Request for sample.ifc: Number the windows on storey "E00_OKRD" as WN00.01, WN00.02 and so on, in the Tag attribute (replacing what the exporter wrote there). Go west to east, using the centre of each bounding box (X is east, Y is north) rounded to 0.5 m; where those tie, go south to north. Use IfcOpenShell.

First a look at what the model holds.

```python
import ifcopenshell
import ifcopenshell.util.element
import ifcopenshell.util.placement

model = ifcopenshell.open("sample.ifc")
print(model.schema)
storey = next(s for s in model.by_type("IfcBuildingStorey") if s.Name == "E00_OKRD")
windows = [e for e in ifcopenshell.util.element.get_decomposition(storey) if e.is_a("IfcWindow")]
for e in sorted(windows, key=lambda e: e.id()):
    origin = ifcopenshell.util.placement.get_local_placement(e.ObjectPlacement)[:3, 3]
    print(e.id(), e.Tag, e.Name, origin.round(2) + 0.0, sep=" | ")
```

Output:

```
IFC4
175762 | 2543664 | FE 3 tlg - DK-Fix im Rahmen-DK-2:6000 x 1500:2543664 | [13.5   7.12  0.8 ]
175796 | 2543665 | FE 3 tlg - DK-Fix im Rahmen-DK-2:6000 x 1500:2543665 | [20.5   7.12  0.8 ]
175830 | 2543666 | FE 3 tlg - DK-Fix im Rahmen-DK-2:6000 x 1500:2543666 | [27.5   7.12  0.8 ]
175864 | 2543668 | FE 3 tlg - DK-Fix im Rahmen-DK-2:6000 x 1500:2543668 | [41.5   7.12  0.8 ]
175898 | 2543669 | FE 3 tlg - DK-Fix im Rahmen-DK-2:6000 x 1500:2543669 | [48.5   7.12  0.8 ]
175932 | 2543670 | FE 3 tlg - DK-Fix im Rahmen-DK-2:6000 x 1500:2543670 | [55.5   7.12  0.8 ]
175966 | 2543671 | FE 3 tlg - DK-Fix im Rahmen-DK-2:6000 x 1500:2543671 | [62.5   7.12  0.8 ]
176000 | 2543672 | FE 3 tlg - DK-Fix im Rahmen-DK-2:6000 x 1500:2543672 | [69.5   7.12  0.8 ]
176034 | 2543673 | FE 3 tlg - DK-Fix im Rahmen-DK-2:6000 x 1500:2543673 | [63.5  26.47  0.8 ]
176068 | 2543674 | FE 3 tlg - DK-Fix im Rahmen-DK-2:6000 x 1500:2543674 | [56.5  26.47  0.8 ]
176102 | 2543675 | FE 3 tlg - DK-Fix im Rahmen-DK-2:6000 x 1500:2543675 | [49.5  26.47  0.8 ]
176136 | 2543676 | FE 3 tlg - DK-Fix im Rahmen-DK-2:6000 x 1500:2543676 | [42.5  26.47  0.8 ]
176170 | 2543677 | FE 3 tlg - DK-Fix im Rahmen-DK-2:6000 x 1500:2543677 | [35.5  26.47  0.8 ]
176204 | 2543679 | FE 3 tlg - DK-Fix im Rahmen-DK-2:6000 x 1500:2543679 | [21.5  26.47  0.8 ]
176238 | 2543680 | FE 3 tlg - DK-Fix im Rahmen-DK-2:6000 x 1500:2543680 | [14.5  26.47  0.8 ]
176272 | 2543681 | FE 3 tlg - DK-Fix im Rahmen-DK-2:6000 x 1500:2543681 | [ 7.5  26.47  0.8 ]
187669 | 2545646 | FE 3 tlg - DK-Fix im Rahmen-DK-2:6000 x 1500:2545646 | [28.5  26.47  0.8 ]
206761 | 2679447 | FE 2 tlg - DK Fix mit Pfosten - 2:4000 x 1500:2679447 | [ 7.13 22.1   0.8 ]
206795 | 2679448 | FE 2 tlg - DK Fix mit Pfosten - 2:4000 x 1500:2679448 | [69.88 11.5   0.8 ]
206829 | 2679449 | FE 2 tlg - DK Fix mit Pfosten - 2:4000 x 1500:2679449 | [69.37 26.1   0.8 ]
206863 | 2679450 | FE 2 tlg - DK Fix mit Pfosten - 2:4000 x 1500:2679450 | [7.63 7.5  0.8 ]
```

```python
import ifcopenshell
import ifcopenshell.geom
import ifcopenshell.util.element
import ifcopenshell.util.shape

model = ifcopenshell.open("sample.ifc")
settings = ifcopenshell.geom.settings()
settings.set("use-world-coords", True)


def centre(element):
    shape = ifcopenshell.geom.create_shape(settings, element)
    return ifcopenshell.util.shape.get_bbox_centroid(shape.geometry)


storey = next(s for s in model.by_type("IfcBuildingStorey") if s.Name == "E00_OKRD")
windows = [e for e in ifcopenshell.util.element.get_decomposition(storey) if e.is_a("IfcWindow")]

# Insertion points can sit at a corner or the storey origin, so sort by the geometry (in metres).
centres = {e: centre(e) for e in windows}
windows.sort(key=lambda e: (round(centres[e][0] / 0.5), centres[e][1]))

for i, e in enumerate(windows, start=1):
    number = f"WN00.{i:02d}"
    e.Tag = number
    print(e.id(), number)

model.write("sample_updated.ifc")
```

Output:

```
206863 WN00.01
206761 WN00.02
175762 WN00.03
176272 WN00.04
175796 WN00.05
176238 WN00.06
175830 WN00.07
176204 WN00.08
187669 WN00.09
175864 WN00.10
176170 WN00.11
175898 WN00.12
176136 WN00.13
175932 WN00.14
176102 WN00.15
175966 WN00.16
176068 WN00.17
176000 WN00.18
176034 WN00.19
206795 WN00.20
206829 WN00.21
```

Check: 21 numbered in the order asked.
